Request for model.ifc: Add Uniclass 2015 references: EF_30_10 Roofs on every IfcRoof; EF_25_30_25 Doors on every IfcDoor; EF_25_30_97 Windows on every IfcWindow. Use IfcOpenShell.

First a look at what the model holds.

```python
import ifcopenshell

model = ifcopenshell.open("model.ifc")
print(model.schema)
print("classifications:", [c.Name for c in model.by_type("IfcClassification")])
for ifc_class in ("IfcDoor", "IfcRoof", "IfcStair", "IfcWall", "IfcWindow"):
    print(ifc_class, len(model.by_type(ifc_class)))
```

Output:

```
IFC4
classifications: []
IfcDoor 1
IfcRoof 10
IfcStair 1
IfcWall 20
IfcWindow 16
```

```python
import ifcopenshell
import ifcopenshell.api.classification

model = ifcopenshell.open("model.ifc")

system = ifcopenshell.api.classification.add_classification(model, classification="Uniclass 2015")

codes = {
    "IfcRoof": ("EF_30_10", "Roofs"),
    "IfcDoor": ("EF_25_30_25", "Doors"),
    "IfcWindow": ("EF_25_30_97", "Windows"),
}
for ifc_class, (code, name) in codes.items():
    products = model.by_type(ifc_class)
    ifcopenshell.api.classification.add_reference(
        model, products=products, classification=system, identification=code, name=name
    )
    print(code, len(products))

model.write("model_rev.ifc")
```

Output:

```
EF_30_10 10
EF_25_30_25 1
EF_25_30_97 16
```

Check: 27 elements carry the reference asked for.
